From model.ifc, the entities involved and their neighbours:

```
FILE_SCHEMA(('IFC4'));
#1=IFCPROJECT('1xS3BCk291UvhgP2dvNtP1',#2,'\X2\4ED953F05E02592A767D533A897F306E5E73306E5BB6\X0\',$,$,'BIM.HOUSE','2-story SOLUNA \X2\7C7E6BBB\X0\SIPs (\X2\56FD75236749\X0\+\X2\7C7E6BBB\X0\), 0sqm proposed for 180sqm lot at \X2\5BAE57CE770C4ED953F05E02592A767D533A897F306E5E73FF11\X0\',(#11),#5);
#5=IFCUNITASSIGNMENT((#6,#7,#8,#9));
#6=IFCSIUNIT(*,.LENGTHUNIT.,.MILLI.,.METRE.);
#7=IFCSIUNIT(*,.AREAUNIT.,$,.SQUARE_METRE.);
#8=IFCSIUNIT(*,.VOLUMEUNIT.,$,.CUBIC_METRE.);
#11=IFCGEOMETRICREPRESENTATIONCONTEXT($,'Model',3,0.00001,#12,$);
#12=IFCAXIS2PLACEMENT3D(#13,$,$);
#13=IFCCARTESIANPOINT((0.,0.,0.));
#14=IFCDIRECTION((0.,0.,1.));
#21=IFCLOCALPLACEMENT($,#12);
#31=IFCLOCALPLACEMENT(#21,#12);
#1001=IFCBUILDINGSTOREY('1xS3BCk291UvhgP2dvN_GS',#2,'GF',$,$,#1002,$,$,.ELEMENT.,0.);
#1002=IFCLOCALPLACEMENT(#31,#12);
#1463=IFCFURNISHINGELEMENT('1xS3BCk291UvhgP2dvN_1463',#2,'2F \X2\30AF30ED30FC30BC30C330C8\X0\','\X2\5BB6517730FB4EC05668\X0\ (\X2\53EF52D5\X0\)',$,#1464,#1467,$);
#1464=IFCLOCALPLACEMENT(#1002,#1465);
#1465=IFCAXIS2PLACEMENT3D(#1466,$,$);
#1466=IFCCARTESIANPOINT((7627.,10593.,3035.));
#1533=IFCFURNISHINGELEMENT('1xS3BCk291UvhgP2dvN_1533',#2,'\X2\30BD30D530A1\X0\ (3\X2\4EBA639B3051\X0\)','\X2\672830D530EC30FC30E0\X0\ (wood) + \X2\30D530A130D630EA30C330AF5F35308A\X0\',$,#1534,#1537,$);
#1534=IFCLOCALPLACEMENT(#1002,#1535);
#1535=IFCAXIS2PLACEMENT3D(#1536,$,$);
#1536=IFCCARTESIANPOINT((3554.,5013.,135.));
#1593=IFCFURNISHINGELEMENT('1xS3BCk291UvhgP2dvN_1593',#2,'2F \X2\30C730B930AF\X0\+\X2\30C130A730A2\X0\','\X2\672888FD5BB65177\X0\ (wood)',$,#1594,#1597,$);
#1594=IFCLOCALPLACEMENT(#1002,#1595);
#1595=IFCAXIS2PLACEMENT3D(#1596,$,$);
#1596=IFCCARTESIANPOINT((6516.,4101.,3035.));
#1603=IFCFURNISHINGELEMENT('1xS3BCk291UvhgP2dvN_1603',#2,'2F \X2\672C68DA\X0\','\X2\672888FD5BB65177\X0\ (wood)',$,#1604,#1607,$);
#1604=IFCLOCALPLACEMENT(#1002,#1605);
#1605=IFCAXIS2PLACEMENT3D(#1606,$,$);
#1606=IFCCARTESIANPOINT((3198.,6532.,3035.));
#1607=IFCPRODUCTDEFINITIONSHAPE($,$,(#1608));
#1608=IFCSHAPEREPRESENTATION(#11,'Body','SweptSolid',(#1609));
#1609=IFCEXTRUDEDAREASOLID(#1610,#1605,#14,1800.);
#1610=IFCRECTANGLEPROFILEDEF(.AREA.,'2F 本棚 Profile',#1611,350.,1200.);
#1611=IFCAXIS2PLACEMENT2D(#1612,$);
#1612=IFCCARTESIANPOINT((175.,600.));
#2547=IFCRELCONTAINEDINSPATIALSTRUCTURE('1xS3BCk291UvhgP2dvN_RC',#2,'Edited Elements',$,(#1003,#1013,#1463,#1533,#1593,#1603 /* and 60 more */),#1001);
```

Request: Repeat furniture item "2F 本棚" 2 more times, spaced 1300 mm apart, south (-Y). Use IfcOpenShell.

```python
import numpy as np
import ifcopenshell
import ifcopenshell.api.geometry
import ifcopenshell.api.root
import ifcopenshell.util.element
import ifcopenshell.util.placement
import ifcopenshell.util.unit

model = ifcopenshell.open("model.ifc")
unit_scale = ifcopenshell.util.unit.calculate_unit_scale(model)


def reuse_history(source, copy):
    """copy_class also copies each property set's owner history, people and application; keep the originals."""
    for rel in copy.IsDefinedBy:
        if rel.is_a("IfcRelDefinesByProperties") and (history := rel.RelatingPropertyDefinition.OwnerHistory):
            rel.RelatingPropertyDefinition.OwnerHistory = source.OwnerHistory
            ifcopenshell.util.element.remove_deep2(model, history)


source = model.by_guid("1xS3BCk291UvhgP2dvN_1603")
base = ifcopenshell.util.placement.get_local_placement(source.ObjectPlacement)
step = np.array([0.0, -1.0, 0.0]) * 1.3 / unit_scale

for i in range(1, 3):
    copy = ifcopenshell.api.root.copy_class(model, product=source)
    copy.Representation = ifcopenshell.util.element.copy_deep(
        model, source.Representation, exclude=["IfcGeometricRepresentationContext", "IfcRepresentationMap"]
    )
    reuse_history(source, copy)
    matrix = base.copy()
    matrix[:3, 3] += i * step
    print("added at", matrix[:3, 3].round(3) + 0.0)
    ifcopenshell.api.geometry.edit_object_placement(model, product=copy, matrix=matrix, is_si=False)

model.write("model_rev.ifc")
```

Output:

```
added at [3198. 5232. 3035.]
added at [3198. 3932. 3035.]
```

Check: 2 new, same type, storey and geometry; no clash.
